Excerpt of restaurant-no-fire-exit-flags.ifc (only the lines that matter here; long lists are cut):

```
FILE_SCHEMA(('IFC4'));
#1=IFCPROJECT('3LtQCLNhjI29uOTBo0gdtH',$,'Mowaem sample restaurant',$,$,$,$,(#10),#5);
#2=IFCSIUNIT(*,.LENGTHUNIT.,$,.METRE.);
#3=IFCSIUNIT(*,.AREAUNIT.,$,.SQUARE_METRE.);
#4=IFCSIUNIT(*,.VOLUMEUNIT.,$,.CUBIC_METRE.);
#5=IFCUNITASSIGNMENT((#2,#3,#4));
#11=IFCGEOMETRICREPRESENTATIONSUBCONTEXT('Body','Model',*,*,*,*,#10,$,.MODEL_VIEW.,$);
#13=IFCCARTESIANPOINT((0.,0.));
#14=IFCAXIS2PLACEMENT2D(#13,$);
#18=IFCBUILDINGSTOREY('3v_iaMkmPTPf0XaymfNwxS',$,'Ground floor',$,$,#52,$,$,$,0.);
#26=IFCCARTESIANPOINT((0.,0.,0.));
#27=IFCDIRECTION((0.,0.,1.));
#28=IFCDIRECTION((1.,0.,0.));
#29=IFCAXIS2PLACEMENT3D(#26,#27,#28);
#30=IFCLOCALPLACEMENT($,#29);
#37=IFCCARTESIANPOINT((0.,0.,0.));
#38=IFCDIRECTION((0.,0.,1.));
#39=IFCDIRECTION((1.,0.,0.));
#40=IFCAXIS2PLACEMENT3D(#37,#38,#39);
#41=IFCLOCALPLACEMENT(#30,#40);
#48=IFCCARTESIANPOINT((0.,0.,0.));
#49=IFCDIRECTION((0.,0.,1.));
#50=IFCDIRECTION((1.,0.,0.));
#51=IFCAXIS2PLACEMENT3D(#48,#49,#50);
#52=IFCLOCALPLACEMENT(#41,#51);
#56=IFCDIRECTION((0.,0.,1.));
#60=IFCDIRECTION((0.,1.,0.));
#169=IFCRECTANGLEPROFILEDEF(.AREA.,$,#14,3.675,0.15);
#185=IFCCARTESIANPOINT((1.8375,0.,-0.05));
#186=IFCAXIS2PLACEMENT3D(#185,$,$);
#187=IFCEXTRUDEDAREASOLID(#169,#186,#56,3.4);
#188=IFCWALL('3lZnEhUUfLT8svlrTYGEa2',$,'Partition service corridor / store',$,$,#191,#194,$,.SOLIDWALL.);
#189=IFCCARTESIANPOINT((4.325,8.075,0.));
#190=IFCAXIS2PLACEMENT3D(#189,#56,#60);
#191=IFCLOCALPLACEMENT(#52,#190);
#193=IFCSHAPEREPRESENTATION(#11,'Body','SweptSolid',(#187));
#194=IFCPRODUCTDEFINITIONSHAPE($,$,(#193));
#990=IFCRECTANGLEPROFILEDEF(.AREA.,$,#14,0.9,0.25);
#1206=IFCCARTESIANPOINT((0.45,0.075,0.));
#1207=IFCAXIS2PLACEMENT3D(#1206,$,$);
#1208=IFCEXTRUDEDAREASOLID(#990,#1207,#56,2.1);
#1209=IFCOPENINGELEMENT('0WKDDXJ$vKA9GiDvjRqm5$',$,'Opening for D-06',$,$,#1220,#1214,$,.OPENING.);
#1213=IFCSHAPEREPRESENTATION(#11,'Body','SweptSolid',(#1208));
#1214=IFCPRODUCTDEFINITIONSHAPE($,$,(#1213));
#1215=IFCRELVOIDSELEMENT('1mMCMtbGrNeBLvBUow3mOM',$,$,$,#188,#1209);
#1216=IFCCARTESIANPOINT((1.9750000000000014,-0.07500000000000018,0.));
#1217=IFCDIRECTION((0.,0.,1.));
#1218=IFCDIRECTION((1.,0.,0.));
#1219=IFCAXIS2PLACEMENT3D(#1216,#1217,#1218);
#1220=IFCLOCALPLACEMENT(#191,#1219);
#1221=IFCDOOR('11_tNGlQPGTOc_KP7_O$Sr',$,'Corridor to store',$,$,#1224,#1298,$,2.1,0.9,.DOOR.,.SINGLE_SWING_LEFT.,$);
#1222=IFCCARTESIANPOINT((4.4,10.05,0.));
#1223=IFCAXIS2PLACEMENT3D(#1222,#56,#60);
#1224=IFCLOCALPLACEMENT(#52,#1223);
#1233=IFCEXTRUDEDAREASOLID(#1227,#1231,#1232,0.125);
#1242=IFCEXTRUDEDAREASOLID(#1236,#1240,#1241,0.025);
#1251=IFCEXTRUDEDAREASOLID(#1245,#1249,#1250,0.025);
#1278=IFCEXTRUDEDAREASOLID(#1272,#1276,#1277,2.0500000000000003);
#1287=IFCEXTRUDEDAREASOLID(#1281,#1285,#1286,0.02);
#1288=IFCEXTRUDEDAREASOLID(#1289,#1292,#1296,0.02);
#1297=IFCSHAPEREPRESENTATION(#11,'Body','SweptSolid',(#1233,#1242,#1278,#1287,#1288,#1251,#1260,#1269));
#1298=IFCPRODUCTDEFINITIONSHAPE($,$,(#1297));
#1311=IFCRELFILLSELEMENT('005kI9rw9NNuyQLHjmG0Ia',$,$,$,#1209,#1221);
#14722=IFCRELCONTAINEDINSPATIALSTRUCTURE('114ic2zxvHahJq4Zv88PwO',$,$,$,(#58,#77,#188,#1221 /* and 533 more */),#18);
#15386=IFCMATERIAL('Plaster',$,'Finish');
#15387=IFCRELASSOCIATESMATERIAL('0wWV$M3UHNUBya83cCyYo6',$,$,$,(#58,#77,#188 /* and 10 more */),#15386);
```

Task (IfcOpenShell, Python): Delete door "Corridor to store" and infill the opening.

```python
import ifcopenshell
import ifcopenshell.api.feature
import ifcopenshell.api.root
import ifcopenshell.geom
import ifcopenshell.util.shape

model = ifcopenshell.open("restaurant-no-fire-exit-flags.ifc")
settings = ifcopenshell.geom.settings()


def volume(element):
    """Net volume in cubic metres, openings subtracted."""
    shape = ifcopenshell.geom.create_shape(settings, element)
    return ifcopenshell.util.shape.get_volume(shape.geometry)


door = model.by_id(1221)
opening = door.FillsVoids[0].RelatingOpeningElement
wall = opening.VoidsElements[0].RelatingBuildingElement
before = volume(wall)

ifcopenshell.api.root.remove_product(model, product=door)
ifcopenshell.api.feature.remove_feature(model, feature=opening)

after = volume(wall)

print(f"wall volume {before:.3f} -> {after:.3f} m3")

model.write("restaurant-no-fire-exit-flags_v2.ifc")
```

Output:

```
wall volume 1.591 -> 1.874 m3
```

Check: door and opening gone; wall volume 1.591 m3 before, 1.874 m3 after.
